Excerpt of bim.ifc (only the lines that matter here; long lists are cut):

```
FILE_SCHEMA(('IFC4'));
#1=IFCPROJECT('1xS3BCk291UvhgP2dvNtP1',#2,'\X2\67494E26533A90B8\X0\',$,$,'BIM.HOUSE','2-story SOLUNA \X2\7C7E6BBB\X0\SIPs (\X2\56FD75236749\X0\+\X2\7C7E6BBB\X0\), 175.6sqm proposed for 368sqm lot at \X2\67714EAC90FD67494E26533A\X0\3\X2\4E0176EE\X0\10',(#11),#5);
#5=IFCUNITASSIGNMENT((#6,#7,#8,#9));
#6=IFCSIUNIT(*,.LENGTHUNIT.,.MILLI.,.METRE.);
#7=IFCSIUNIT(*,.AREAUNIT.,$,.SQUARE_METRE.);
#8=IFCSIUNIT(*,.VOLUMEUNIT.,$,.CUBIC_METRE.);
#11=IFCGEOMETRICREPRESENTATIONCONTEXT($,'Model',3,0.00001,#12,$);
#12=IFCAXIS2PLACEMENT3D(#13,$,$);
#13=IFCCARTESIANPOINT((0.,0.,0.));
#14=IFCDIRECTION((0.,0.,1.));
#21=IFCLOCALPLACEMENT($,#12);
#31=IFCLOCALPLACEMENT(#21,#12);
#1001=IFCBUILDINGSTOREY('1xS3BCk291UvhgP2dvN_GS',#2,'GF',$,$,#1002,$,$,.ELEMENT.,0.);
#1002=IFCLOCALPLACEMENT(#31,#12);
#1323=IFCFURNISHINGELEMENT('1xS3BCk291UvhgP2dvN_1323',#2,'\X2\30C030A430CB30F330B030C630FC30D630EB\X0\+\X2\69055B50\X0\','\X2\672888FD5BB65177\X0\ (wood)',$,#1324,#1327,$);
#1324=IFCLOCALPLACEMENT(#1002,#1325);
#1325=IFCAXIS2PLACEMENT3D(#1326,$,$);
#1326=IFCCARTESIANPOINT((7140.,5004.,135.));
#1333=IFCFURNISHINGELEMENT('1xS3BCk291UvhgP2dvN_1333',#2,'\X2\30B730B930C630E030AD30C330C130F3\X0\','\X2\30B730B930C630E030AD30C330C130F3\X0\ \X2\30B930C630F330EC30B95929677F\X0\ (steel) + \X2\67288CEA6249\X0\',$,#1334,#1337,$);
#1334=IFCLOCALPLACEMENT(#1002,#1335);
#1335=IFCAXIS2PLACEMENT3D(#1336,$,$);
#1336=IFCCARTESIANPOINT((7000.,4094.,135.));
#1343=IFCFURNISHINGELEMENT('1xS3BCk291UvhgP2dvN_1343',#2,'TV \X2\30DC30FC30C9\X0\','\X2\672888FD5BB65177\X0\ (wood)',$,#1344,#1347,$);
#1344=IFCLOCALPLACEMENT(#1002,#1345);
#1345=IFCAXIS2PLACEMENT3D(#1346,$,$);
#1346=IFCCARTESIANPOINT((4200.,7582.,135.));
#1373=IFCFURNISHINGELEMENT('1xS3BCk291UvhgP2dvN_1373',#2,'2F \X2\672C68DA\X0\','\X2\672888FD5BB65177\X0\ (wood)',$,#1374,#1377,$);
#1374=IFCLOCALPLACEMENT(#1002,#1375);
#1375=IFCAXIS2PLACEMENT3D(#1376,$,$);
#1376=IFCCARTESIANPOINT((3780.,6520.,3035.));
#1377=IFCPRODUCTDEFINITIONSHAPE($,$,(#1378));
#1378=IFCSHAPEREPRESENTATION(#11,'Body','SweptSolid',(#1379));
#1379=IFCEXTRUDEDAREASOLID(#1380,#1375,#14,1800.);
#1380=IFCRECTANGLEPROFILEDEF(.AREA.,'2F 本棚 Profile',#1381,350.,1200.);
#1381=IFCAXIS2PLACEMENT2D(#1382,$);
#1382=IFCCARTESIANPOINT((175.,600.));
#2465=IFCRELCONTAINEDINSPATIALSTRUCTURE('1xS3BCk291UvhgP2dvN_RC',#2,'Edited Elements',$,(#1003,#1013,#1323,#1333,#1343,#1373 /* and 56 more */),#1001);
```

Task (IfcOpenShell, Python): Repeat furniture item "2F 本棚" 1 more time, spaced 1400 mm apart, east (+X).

```python
import numpy as np
import ifcopenshell
import ifcopenshell.api.geometry
import ifcopenshell.api.root
import ifcopenshell.util.element
import ifcopenshell.util.placement
import ifcopenshell.util.unit

model = ifcopenshell.open("bim.ifc")
unit_scale = ifcopenshell.util.unit.calculate_unit_scale(model)


def reuse_history(source, copy):
    """copy_class also copies each property set's owner history, people and application; keep the originals."""
    for rel in copy.IsDefinedBy:
        if rel.is_a("IfcRelDefinesByProperties") and (history := rel.RelatingPropertyDefinition.OwnerHistory):
            rel.RelatingPropertyDefinition.OwnerHistory = source.OwnerHistory
            ifcopenshell.util.element.remove_deep2(model, history)


source = model.by_guid("1xS3BCk291UvhgP2dvN_1373")
base = ifcopenshell.util.placement.get_local_placement(source.ObjectPlacement)
step = np.array([1.0, 0.0, 0.0]) * 1.4 / unit_scale

for i in range(1, 2):
    copy = ifcopenshell.api.root.copy_class(model, product=source)
    copy.Representation = ifcopenshell.util.element.copy_deep(
        model, source.Representation, exclude=["IfcGeometricRepresentationContext", "IfcRepresentationMap"]
    )
    reuse_history(source, copy)
    matrix = base.copy()
    matrix[:3, 3] += i * step
    print("added at", matrix[:3, 3].round(3) + 0.0)
    ifcopenshell.api.geometry.edit_object_placement(model, product=copy, matrix=matrix, is_si=False)

model.write("bim_edited.ifc")
```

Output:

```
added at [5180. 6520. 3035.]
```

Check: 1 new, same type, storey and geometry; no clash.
